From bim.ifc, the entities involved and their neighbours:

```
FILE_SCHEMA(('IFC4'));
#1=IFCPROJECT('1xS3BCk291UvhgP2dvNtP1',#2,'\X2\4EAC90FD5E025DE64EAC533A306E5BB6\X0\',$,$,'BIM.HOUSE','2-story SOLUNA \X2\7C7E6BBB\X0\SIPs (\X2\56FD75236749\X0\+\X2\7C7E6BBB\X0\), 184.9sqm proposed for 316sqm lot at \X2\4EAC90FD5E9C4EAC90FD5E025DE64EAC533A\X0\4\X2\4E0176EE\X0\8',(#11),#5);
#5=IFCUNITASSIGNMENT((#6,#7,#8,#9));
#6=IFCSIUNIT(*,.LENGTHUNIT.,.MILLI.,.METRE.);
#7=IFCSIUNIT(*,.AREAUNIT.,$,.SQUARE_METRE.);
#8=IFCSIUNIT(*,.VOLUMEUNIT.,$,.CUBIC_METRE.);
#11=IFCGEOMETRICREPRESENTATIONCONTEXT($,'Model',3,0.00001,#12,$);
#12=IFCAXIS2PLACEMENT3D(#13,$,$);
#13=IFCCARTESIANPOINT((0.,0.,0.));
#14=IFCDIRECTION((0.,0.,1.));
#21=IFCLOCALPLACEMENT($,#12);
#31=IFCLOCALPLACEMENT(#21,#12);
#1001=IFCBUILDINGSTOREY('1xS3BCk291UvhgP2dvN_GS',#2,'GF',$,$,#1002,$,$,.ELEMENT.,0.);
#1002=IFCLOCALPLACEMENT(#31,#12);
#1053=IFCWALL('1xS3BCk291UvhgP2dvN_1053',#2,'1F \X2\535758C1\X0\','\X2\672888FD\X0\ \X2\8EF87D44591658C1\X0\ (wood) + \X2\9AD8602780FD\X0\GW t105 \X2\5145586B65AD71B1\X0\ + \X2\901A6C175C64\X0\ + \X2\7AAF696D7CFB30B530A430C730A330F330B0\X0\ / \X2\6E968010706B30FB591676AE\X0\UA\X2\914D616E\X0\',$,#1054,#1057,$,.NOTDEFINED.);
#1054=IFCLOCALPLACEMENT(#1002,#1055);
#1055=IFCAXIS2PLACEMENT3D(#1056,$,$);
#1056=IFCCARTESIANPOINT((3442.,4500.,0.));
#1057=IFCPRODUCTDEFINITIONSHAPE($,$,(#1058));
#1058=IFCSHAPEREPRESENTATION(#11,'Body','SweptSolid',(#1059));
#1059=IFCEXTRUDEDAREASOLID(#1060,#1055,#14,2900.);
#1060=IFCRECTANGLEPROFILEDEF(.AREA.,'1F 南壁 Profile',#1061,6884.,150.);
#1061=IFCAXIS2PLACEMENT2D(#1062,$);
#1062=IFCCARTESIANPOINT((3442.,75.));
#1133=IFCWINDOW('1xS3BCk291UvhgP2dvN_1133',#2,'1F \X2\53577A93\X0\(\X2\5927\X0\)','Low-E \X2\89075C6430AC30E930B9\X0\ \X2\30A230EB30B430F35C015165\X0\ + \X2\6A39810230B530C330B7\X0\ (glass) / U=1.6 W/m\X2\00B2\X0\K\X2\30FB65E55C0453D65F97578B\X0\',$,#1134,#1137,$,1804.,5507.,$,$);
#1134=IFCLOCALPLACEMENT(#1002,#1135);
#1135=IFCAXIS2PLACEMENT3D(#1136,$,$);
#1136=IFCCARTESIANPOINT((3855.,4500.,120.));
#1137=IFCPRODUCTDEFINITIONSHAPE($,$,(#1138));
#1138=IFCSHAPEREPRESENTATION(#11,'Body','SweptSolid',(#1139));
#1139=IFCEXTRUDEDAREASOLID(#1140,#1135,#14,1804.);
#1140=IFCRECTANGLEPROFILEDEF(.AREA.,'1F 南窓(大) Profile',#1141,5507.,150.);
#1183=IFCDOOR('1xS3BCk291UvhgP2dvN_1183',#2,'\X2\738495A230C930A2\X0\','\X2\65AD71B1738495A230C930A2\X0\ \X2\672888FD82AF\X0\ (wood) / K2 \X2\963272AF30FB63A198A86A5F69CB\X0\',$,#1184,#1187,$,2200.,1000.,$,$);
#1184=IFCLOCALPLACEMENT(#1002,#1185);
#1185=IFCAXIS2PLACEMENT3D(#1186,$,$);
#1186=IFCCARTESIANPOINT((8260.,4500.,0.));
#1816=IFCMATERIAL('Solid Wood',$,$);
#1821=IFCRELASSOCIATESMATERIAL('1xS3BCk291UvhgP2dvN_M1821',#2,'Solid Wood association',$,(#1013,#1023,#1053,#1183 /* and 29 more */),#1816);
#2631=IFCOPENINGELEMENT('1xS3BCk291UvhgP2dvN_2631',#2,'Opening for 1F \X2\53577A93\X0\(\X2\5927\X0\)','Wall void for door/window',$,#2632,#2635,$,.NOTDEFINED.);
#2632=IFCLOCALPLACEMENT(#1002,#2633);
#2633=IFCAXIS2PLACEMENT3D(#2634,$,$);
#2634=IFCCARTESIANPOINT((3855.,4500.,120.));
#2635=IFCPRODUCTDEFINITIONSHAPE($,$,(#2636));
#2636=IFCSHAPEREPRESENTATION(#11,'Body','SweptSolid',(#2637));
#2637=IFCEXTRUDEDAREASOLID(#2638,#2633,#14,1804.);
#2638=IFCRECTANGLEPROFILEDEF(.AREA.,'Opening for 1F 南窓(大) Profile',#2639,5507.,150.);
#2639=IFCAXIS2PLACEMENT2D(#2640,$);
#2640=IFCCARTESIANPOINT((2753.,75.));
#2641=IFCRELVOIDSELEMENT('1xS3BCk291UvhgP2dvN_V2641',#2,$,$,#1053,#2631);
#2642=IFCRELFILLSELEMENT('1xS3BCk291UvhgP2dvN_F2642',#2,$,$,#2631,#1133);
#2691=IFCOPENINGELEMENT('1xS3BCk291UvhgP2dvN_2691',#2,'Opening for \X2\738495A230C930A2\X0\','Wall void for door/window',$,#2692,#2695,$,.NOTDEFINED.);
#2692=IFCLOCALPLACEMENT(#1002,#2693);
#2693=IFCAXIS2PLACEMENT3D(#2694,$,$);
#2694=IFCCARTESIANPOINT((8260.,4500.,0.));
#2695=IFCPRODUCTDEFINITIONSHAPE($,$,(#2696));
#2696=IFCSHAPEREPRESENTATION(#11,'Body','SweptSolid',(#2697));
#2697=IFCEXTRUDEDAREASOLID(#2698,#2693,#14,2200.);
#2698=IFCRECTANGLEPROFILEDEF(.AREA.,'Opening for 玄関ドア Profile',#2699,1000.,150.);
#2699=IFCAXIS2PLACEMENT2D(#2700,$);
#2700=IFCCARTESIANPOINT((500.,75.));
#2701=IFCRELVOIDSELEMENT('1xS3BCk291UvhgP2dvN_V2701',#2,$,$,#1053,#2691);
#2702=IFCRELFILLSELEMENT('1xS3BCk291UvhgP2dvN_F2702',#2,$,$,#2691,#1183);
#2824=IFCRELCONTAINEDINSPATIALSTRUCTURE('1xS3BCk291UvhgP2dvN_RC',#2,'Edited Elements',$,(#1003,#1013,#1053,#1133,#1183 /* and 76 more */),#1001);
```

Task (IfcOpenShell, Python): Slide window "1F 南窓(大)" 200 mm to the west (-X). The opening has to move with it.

```python
import ifcopenshell
import ifcopenshell.api.geometry
import ifcopenshell.util.placement
import ifcopenshell.util.unit

model = ifcopenshell.open("bim.ifc")
unit_scale = ifcopenshell.util.unit.calculate_unit_scale(model)

window = model.by_guid("1xS3BCk291UvhgP2dvN_1133")
opening = window.FillsVoids[0].RelatingOpeningElement
wall = opening.VoidsElements[0].RelatingBuildingElement

wall_matrix = ifcopenshell.util.placement.get_local_placement(wall.ObjectPlacement)
shift = wall_matrix[:3, 0] * -0.2 / unit_scale
before = ifcopenshell.util.placement.get_local_placement(window.ObjectPlacement)[:3, 3].copy()

# The window is not placed relative to its opening, so move both.
for product in (opening, window):
    matrix = ifcopenshell.util.placement.get_local_placement(product.ObjectPlacement)
    matrix[:3, 3] += shift
    ifcopenshell.api.geometry.edit_object_placement(model, product=product, matrix=matrix, is_si=False)

after = ifcopenshell.util.placement.get_local_placement(window.ObjectPlacement)[:3, 3]
print("window moved by", (after - before).round(3) + 0.0)

model.write("bim-out.ifc")
```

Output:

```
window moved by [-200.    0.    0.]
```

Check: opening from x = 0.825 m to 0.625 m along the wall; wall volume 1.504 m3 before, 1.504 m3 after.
